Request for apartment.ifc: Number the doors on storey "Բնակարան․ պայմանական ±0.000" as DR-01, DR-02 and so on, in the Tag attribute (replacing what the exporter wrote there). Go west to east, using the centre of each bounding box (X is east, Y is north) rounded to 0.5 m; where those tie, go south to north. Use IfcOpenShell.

First a look at what the model holds.

```python
import ifcopenshell
import ifcopenshell.util.element
import ifcopenshell.util.placement

model = ifcopenshell.open("apartment.ifc")
print(model.schema)
storey = next(s for s in model.by_type("IfcBuildingStorey") if s.Name == "Բնակարան․ պայմանական ±0.000")
doors = [e for e in ifcopenshell.util.element.get_decomposition(storey) if e.is_a("IfcDoor")]
for e in sorted(doors, key=lambda e: e.id()):
    origin = ifcopenshell.util.placement.get_local_placement(e.ObjectPlacement)[:3, 3]
    print(e.id(), e.Tag, e.Name, origin.round(2) + 0.0, sep=" | ")
```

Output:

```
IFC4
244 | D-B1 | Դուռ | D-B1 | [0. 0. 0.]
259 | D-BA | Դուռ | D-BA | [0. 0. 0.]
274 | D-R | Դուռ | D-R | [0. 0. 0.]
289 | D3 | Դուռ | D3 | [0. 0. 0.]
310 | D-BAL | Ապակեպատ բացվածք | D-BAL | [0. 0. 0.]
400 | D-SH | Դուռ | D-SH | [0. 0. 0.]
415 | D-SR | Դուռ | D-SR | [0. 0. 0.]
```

```python
import ifcopenshell
import ifcopenshell.geom
import ifcopenshell.util.element
import ifcopenshell.util.shape

model = ifcopenshell.open("apartment.ifc")
settings = ifcopenshell.geom.settings()
settings.set("use-world-coords", True)


def centre(element):
    shape = ifcopenshell.geom.create_shape(settings, element)
    return ifcopenshell.util.shape.get_bbox_centroid(shape.geometry)


storey = next(s for s in model.by_type("IfcBuildingStorey") if s.Name == "Բնակարան․ պայմանական ±0.000")
doors = [e for e in ifcopenshell.util.element.get_decomposition(storey) if e.is_a("IfcDoor")]

# Insertion points can sit at a corner or the storey origin, so sort by the geometry (in metres).
centres = {e: centre(e) for e in doors}
doors.sort(key=lambda e: (round(centres[e][0] / 0.5), centres[e][1]))

for i, e in enumerate(doors, start=1):
    number = f"DR-{i:02d}"
    e.Tag = number
    print(e.id(), number)

model.write("apartment_rev.ifc")
```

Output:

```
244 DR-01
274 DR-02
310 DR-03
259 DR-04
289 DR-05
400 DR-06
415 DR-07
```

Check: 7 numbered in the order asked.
